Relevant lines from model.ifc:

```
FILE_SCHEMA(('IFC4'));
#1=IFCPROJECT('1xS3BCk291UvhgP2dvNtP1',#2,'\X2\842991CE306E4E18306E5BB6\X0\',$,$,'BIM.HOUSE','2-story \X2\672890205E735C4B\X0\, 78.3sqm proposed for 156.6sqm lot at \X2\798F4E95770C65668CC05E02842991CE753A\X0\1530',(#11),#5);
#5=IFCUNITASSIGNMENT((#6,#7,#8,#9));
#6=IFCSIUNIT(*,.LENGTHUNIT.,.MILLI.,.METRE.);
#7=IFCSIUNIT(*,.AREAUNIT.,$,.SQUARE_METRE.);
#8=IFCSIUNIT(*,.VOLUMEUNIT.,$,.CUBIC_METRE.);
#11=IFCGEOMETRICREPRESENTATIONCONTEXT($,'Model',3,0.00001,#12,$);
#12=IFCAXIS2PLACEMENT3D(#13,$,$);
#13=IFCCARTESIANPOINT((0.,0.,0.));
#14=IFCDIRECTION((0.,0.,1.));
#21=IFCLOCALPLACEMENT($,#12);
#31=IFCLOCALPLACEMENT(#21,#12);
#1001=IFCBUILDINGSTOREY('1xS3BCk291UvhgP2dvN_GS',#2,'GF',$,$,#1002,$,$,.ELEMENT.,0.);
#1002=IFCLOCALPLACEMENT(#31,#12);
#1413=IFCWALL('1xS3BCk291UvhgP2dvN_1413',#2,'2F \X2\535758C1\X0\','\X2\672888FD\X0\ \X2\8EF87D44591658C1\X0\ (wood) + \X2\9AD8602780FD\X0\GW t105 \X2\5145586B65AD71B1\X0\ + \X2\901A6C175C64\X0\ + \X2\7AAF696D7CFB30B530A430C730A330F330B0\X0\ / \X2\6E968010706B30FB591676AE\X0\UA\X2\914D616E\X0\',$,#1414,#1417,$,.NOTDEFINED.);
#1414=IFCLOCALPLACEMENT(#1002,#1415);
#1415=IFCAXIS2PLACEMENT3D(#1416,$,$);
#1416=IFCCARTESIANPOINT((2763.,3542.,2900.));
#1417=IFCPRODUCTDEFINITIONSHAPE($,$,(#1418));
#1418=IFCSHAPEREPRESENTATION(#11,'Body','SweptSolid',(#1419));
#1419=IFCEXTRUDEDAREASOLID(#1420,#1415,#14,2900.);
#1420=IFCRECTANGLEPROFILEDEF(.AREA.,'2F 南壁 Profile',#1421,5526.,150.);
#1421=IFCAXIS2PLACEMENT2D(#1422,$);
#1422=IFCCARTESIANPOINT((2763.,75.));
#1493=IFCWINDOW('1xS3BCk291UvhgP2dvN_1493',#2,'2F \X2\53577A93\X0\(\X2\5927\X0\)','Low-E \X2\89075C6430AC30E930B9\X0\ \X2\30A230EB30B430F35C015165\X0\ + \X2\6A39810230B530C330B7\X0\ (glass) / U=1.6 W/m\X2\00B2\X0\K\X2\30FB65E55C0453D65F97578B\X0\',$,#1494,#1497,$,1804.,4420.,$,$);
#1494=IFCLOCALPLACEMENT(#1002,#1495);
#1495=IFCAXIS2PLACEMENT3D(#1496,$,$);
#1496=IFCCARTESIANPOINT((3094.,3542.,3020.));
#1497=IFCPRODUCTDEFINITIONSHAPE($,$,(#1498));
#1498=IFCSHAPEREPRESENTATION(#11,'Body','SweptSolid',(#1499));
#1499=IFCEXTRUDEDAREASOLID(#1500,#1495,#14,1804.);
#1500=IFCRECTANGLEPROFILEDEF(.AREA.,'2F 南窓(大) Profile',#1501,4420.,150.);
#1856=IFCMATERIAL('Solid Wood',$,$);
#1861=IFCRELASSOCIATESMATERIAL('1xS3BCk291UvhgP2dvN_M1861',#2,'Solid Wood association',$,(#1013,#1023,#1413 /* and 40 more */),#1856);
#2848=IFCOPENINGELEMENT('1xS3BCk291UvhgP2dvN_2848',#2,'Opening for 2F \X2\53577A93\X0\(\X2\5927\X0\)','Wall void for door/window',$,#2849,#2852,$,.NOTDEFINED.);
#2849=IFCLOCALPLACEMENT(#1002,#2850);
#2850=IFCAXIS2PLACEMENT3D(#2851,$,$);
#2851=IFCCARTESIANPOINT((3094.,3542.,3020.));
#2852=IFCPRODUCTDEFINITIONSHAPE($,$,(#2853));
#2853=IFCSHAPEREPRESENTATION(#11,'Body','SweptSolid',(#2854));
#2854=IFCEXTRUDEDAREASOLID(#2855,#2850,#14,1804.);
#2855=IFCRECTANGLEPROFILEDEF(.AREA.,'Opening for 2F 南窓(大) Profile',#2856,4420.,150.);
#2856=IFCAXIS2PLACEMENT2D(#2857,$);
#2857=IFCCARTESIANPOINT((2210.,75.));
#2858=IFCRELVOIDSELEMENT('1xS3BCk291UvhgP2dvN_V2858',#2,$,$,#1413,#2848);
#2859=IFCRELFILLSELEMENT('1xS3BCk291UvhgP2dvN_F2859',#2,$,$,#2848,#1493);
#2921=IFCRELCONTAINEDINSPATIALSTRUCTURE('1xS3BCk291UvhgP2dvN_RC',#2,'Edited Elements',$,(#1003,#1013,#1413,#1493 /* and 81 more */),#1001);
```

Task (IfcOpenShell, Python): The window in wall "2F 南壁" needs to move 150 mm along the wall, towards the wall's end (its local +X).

```python
import ifcopenshell
import ifcopenshell.api.geometry
import ifcopenshell.util.placement
import ifcopenshell.util.unit

model = ifcopenshell.open("model.ifc")
unit_scale = ifcopenshell.util.unit.calculate_unit_scale(model)

window = model.by_id(1493)
opening = window.FillsVoids[0].RelatingOpeningElement
wall = opening.VoidsElements[0].RelatingBuildingElement

wall_matrix = ifcopenshell.util.placement.get_local_placement(wall.ObjectPlacement)
shift = wall_matrix[:3, 0] * 0.15 / unit_scale
before = ifcopenshell.util.placement.get_local_placement(window.ObjectPlacement)[:3, 3].copy()

# The window is not placed relative to its opening, so move both.
for product in (opening, window):
    matrix = ifcopenshell.util.placement.get_local_placement(product.ObjectPlacement)
    matrix[:3, 3] += shift
    ifcopenshell.api.geometry.edit_object_placement(model, product=product, matrix=matrix, is_si=False)

after = ifcopenshell.util.placement.get_local_placement(window.ObjectPlacement)[:3, 3]
print("window moved by", (after - before).round(3) + 0.0)

model.write("model_v2.ifc")
```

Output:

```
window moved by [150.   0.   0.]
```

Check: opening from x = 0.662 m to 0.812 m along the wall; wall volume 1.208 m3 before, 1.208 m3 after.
